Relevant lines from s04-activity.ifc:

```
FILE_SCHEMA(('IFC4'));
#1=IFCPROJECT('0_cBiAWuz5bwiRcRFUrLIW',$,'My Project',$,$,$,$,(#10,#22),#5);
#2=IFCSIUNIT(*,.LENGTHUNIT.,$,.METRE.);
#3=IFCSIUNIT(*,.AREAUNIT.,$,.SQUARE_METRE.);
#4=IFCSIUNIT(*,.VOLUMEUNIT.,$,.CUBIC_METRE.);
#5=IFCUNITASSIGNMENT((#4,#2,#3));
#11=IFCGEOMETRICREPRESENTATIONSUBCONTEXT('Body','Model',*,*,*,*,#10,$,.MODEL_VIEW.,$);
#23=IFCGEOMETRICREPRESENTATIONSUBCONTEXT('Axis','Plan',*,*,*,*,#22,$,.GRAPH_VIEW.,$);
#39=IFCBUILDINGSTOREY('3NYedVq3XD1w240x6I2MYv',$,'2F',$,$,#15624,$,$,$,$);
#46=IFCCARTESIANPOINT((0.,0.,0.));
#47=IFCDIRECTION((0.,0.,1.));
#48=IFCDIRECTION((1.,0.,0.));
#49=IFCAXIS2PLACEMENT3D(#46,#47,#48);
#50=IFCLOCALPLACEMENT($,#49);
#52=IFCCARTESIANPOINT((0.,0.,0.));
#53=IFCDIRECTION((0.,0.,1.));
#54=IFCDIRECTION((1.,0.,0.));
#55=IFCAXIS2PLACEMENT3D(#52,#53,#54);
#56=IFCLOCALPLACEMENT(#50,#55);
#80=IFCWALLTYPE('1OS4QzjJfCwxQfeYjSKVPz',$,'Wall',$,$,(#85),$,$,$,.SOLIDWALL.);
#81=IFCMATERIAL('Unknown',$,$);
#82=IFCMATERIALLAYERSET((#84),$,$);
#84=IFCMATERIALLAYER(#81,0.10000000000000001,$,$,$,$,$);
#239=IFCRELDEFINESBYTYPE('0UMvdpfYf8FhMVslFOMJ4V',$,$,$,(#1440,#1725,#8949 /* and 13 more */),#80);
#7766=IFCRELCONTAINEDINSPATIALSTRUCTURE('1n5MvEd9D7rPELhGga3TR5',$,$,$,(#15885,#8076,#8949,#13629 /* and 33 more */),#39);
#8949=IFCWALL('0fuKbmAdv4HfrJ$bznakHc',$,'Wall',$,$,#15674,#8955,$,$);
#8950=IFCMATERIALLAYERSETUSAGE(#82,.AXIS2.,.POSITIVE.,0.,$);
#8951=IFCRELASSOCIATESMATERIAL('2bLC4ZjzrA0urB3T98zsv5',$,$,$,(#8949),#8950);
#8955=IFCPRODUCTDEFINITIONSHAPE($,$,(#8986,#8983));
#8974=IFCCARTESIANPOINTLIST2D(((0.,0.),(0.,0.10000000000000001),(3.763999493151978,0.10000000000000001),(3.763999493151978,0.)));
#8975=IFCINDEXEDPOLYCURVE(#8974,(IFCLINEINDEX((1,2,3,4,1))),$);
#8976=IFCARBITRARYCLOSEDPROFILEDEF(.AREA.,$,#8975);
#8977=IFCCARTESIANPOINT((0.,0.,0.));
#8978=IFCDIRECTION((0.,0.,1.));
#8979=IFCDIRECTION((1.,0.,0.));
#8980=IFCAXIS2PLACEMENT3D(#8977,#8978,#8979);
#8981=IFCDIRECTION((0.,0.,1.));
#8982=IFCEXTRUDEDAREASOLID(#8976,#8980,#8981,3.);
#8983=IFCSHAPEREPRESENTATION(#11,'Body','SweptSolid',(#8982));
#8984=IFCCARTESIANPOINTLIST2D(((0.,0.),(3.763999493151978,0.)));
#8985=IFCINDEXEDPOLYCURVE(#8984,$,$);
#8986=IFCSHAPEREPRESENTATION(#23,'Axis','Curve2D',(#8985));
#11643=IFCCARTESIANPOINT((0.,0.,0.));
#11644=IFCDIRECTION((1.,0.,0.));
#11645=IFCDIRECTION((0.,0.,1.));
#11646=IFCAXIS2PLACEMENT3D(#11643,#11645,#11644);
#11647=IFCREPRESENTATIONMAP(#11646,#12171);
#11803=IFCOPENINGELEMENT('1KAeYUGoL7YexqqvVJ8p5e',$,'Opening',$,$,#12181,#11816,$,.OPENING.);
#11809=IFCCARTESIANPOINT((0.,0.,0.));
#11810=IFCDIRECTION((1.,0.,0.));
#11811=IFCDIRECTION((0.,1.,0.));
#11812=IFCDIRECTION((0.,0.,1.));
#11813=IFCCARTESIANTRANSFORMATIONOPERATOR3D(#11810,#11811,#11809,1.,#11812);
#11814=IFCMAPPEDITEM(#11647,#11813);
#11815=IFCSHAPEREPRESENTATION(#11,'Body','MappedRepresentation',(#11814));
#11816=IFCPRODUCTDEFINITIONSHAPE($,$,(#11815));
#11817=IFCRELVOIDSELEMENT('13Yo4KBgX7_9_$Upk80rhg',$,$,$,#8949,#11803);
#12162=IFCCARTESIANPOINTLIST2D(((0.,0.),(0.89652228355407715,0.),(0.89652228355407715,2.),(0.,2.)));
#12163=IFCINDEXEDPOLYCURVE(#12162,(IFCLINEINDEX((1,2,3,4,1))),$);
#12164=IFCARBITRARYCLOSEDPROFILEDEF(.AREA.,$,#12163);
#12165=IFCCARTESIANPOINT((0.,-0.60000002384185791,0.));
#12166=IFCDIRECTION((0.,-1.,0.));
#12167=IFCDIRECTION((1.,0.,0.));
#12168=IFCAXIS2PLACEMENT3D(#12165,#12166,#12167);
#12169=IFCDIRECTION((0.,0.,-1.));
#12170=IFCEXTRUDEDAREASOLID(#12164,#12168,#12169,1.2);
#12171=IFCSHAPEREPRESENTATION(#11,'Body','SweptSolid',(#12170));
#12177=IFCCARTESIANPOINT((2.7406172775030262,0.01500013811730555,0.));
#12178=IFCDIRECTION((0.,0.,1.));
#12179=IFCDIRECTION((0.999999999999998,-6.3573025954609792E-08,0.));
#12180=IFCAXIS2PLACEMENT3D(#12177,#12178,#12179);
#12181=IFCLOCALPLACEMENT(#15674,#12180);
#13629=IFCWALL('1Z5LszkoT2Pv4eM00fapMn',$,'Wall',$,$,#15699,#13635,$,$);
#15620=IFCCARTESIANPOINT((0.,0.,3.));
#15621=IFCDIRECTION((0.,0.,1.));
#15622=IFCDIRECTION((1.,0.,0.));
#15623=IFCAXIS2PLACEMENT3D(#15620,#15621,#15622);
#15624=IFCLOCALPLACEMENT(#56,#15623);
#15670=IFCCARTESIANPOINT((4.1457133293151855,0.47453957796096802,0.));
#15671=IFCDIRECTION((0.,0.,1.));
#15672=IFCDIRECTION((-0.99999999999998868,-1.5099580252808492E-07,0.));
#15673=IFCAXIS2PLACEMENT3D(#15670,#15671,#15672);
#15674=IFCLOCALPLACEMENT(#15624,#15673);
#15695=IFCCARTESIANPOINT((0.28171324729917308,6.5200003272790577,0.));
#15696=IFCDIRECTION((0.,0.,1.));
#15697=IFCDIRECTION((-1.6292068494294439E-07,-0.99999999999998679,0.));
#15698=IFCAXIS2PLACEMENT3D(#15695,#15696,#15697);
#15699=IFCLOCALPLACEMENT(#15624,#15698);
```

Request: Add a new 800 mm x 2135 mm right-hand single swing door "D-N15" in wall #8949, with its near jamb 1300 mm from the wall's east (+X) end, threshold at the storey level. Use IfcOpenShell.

```python
import numpy as np
import ifcopenshell
import ifcopenshell.api.feature
import ifcopenshell.api.geometry
import ifcopenshell.api.root
import ifcopenshell.api.spatial
import ifcopenshell.geom
import ifcopenshell.util.element
import ifcopenshell.util.placement
import ifcopenshell.util.representation
import ifcopenshell.util.shape
import ifcopenshell.util.unit

model = ifcopenshell.open("s04-activity.ifc")
unit_scale = ifcopenshell.util.unit.calculate_unit_scale(model)
settings = ifcopenshell.geom.settings()


def volume(element):
    """Net volume in cubic metres, openings subtracted."""
    shape = ifcopenshell.geom.create_shape(settings, element)
    return ifcopenshell.util.shape.get_volume(shape.geometry)


wall = model.by_guid("0fuKbmAdv4HfrJ$bznakHc")
storey = ifcopenshell.util.element.get_container(wall, ifc_class="IfcBuildingStorey")
context = ifcopenshell.util.representation.get_context(model, "Model", "Body", "MODEL_VIEW")
before = volume(wall)

width, height, from_end, sill = 0.8, 2.135, 1.3, 0.0  # metres

# The wall runs along its own X axis, and the end named is its -X end.
wall_shape = ifcopenshell.geom.create_shape(settings, wall)
x, y, z = ifcopenshell.util.shape.get_vertices(wall_shape.geometry).T
start = x.min() + from_end
face, thickness = float(y.min()), float(y.max() - y.min())
wall_matrix = ifcopenshell.util.placement.get_local_placement(wall.ObjectPlacement)
level = ifcopenshell.util.placement.get_local_placement(storey.ObjectPlacement)[2, 3]


def in_wall(x, y):
    """Placement at x, y metres in the wall's axes, at sill height."""
    matrix = wall_matrix.copy()
    matrix[:, 3] = wall_matrix @ np.array([x / unit_scale, y / unit_scale, 0.0, 1.0])
    matrix[2, 3] = level + sill / unit_scale
    return matrix


# Opening: a box that overshoots both wall faces by 50 mm.
opening = ifcopenshell.api.root.create_entity(model, ifc_class="IfcOpeningElement", predefined_type="OPENING")
box = ifcopenshell.api.geometry.add_wall_representation(
    model, context=context, length=width, height=height, thickness=thickness + 0.1
)
ifcopenshell.api.geometry.assign_representation(model, product=opening, representation=box)
ifcopenshell.api.geometry.edit_object_placement(model, product=opening, matrix=in_wall(start, face - 0.05), is_si=False)
ifcopenshell.api.feature.add_feature(model, feature=opening, element=wall)

door = ifcopenshell.api.root.create_entity(model, ifc_class="IfcDoor", name="D-N15", predefined_type="DOOR")
door.OverallWidth, door.OverallHeight = width / unit_scale, height / unit_scale
door.OperationType = "SINGLE_SWING_RIGHT"
body = ifcopenshell.api.geometry.add_door_representation(
    model,
    context=context,
    overall_width=door.OverallWidth,
    overall_height=door.OverallHeight,
    operation_type="SINGLE_SWING_RIGHT",
    lining_properties={"LiningDepth": thickness / unit_scale, "ThresholdDepth": thickness / unit_scale},
)
ifcopenshell.api.geometry.assign_representation(model, product=door, representation=body)
ifcopenshell.api.spatial.assign_container(model, products=[door], relating_structure=storey)
ifcopenshell.api.feature.add_filling(model, opening=opening, element=door)

# The lining spans the wall, so the door starts at the wall face.
ifcopenshell.api.geometry.edit_object_placement(model, product=door, matrix=in_wall(start, face), is_si=False)

after = volume(wall)

print(f"wall volume {before:.3f} -> {after:.3f} m3")

model.write("s04-activity_v2.ifc")
```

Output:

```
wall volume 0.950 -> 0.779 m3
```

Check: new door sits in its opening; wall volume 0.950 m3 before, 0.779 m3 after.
